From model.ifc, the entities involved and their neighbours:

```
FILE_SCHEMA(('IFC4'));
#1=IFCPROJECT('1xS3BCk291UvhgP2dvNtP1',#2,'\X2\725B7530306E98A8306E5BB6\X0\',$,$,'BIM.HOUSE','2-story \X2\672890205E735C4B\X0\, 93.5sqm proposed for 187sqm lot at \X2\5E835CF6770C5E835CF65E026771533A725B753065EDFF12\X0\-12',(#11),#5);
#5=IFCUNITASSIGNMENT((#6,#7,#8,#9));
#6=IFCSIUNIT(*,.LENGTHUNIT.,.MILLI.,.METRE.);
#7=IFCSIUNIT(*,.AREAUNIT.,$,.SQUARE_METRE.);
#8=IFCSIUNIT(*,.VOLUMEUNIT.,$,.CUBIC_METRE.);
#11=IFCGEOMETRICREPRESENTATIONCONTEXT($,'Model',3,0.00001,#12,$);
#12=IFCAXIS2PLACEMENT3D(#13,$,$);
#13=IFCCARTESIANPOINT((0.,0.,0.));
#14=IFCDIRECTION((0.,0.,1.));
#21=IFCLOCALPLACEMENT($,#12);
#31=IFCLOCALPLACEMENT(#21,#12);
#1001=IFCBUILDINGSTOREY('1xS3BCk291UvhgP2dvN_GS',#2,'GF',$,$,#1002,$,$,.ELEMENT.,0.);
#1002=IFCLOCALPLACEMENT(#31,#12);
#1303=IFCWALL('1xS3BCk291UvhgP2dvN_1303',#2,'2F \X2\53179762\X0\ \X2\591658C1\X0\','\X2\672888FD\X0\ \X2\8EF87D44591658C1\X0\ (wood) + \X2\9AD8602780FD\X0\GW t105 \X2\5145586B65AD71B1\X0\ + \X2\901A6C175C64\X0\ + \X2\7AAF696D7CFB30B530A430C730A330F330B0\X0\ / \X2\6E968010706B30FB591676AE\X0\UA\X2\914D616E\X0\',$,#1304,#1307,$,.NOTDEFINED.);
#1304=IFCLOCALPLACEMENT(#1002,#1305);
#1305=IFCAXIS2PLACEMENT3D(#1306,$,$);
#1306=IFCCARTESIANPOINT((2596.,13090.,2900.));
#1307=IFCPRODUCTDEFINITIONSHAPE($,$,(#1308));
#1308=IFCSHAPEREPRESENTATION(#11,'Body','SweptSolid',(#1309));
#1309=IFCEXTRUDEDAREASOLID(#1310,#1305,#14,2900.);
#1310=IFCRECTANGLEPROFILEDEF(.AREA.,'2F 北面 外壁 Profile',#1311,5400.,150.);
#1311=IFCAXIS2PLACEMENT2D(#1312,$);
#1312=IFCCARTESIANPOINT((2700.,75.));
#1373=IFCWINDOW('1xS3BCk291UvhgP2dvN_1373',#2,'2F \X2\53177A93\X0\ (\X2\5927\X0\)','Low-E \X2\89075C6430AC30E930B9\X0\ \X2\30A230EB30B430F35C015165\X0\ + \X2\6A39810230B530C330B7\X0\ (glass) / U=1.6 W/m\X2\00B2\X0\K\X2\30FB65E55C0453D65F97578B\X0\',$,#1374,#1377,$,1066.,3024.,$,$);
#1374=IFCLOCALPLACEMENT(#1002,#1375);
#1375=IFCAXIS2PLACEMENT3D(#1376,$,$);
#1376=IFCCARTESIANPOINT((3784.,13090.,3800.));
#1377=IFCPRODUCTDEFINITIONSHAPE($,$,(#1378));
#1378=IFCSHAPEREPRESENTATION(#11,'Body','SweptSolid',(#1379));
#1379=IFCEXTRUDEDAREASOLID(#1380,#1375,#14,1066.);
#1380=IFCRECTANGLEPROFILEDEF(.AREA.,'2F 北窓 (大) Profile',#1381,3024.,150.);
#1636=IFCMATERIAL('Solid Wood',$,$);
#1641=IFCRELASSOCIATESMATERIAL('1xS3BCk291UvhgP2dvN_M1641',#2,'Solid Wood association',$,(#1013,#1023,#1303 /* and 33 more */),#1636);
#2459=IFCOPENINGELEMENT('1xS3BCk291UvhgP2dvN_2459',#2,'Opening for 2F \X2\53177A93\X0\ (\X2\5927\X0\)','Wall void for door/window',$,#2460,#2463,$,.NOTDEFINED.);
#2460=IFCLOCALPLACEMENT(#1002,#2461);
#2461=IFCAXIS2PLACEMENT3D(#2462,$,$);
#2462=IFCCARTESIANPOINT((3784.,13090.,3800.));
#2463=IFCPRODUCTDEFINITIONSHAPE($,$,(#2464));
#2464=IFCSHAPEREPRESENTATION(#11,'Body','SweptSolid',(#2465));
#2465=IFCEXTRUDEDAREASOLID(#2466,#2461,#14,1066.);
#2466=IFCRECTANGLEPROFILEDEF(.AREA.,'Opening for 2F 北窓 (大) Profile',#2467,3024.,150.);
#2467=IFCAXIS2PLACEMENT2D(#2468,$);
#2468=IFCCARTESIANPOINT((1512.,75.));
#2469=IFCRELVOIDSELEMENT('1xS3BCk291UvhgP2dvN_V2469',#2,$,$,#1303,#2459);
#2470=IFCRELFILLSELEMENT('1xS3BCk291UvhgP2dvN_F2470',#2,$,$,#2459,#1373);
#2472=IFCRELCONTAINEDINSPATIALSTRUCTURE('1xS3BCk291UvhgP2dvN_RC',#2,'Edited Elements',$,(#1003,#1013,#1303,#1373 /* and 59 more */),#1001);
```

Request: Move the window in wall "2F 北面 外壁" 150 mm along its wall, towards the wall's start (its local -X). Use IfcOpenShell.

```python
import ifcopenshell
import ifcopenshell.api.geometry
import ifcopenshell.util.placement
import ifcopenshell.util.unit

model = ifcopenshell.open("model.ifc")
unit_scale = ifcopenshell.util.unit.calculate_unit_scale(model)

window = model.by_guid("1xS3BCk291UvhgP2dvN_1373")
opening = window.FillsVoids[0].RelatingOpeningElement
wall = opening.VoidsElements[0].RelatingBuildingElement

wall_matrix = ifcopenshell.util.placement.get_local_placement(wall.ObjectPlacement)
shift = wall_matrix[:3, 0] * -0.15 / unit_scale
before = ifcopenshell.util.placement.get_local_placement(window.ObjectPlacement)[:3, 3].copy()

# The window is not placed relative to its opening, so move both.
for product in (opening, window):
    matrix = ifcopenshell.util.placement.get_local_placement(product.ObjectPlacement)
    matrix[:3, 3] += shift
    ifcopenshell.api.geometry.edit_object_placement(model, product=product, matrix=matrix, is_si=False)

after = ifcopenshell.util.placement.get_local_placement(window.ObjectPlacement)[:3, 3]
print("window moved by", (after - before).round(3) + 0.0)

model.write("model_rev.ifc")
```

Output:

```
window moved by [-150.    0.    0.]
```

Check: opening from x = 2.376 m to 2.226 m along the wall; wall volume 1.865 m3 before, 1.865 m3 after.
